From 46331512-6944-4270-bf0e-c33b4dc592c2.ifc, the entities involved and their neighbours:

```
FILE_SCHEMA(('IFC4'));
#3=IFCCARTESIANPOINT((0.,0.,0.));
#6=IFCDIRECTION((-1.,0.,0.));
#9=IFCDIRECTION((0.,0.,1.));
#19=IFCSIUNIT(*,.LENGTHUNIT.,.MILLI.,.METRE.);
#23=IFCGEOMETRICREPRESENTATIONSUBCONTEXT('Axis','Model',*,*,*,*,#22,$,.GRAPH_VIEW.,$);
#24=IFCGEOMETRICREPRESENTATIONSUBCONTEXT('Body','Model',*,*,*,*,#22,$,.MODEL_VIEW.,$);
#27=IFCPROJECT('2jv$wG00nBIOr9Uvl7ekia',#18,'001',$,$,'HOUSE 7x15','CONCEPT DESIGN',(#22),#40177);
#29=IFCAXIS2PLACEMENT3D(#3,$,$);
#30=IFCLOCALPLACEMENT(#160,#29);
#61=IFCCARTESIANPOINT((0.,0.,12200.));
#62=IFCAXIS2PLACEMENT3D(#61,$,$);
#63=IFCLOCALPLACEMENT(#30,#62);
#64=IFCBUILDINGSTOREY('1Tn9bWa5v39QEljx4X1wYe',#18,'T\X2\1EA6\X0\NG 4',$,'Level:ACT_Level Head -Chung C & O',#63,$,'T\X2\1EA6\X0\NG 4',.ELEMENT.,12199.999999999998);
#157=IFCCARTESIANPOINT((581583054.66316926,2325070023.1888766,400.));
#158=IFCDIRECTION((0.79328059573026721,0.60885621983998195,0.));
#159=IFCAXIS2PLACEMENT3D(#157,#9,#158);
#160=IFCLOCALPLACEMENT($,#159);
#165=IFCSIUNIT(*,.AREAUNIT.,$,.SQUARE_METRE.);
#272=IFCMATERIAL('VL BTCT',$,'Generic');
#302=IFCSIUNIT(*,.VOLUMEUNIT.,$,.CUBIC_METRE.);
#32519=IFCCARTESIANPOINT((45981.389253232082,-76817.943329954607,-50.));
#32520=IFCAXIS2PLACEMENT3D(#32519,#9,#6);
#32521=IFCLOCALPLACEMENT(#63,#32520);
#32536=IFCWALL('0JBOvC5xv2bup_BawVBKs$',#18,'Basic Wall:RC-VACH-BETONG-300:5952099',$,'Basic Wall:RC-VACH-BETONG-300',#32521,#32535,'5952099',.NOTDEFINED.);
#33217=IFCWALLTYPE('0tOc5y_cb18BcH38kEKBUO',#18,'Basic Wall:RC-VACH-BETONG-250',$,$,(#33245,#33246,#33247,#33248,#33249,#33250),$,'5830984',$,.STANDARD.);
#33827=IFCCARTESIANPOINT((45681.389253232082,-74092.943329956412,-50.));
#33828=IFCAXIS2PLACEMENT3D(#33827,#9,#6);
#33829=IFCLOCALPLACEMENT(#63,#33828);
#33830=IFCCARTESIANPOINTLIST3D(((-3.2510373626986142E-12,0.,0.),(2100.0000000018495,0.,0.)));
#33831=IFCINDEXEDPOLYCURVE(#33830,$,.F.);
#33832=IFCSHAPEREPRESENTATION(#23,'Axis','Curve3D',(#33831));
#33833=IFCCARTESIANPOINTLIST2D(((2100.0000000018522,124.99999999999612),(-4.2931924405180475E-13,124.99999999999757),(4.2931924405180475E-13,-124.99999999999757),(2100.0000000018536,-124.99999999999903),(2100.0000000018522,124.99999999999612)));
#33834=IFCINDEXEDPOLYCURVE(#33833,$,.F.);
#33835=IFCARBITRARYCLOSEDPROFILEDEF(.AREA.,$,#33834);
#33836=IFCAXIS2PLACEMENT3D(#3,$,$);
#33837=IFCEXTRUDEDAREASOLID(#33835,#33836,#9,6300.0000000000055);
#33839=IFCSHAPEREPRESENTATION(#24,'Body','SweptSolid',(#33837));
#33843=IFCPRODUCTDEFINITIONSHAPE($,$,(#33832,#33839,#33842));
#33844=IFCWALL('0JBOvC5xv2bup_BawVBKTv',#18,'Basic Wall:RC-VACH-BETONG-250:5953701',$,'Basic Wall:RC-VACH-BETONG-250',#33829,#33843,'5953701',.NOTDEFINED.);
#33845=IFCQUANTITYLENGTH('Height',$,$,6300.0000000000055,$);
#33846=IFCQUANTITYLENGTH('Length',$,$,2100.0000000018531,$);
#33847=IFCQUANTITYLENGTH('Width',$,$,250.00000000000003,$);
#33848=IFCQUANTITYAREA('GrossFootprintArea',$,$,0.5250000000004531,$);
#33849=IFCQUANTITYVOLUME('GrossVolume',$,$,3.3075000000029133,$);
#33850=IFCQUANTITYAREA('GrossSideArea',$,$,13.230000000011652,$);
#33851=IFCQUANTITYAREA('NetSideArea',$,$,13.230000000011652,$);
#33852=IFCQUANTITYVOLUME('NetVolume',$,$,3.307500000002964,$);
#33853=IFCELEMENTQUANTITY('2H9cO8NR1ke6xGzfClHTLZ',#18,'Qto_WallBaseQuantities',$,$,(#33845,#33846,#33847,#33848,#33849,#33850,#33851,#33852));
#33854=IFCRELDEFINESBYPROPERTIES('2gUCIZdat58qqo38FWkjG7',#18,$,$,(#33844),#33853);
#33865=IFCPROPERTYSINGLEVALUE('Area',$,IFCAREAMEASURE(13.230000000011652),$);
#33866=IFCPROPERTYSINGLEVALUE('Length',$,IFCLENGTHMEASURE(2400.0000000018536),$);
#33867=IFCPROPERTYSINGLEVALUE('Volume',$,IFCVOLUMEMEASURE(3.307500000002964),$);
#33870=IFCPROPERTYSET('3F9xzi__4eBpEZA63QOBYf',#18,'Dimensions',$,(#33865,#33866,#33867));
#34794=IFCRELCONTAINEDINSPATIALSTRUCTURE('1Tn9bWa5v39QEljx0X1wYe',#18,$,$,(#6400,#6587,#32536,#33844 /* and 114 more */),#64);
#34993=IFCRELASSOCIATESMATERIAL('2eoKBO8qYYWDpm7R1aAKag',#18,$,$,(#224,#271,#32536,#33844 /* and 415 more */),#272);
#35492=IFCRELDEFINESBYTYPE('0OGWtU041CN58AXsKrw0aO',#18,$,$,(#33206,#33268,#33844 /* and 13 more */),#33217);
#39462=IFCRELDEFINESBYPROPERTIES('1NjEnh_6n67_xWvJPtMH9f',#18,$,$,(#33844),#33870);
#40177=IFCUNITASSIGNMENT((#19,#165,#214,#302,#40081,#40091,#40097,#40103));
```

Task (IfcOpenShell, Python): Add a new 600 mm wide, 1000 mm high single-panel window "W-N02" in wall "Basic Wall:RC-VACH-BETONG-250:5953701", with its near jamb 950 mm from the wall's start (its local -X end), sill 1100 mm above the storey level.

```python
import numpy as np
import ifcopenshell
import ifcopenshell.api.feature
import ifcopenshell.api.geometry
import ifcopenshell.api.pset
import ifcopenshell.api.root
import ifcopenshell.api.spatial
import ifcopenshell.geom
import ifcopenshell.util.element
import ifcopenshell.util.placement
import ifcopenshell.util.representation
import ifcopenshell.util.shape
import ifcopenshell.util.unit

model = ifcopenshell.open("46331512-6944-4270-bf0e-c33b4dc592c2.ifc")
unit_scale = ifcopenshell.util.unit.calculate_unit_scale(model)
area_scale = ifcopenshell.util.unit.calculate_unit_scale(model, "AREAUNIT")
volume_scale = ifcopenshell.util.unit.calculate_unit_scale(model, "VOLUMEUNIT")
settings = ifcopenshell.geom.settings()


def volume(element):
    """Net volume in cubic metres, openings subtracted."""
    shape = ifcopenshell.geom.create_shape(settings, element)
    return ifcopenshell.util.shape.get_volume(shape.geometry)


wall = model.by_id(33844)
storey = ifcopenshell.util.element.get_container(wall, ifc_class="IfcBuildingStorey")
context = ifcopenshell.util.representation.get_context(model, "Model", "Body", "MODEL_VIEW")
before = volume(wall)

width, height, from_end, sill = 0.6, 1, 0.95, 1.1  # metres

# The wall runs along its own X axis, and the end named is its -X end.
wall_shape = ifcopenshell.geom.create_shape(settings, wall)
x, y, z = ifcopenshell.util.shape.get_vertices(wall_shape.geometry).T
start = x.min() + from_end
face, thickness = float(y.min()), float(y.max() - y.min())
wall_matrix = ifcopenshell.util.placement.get_local_placement(wall.ObjectPlacement)
level = ifcopenshell.util.placement.get_local_placement(storey.ObjectPlacement)[2, 3]


def in_wall(x, y):
    """Placement at x, y metres in the wall's axes, at sill height."""
    matrix = wall_matrix.copy()
    matrix[:, 3] = wall_matrix @ np.array([x / unit_scale, y / unit_scale, 0.0, 1.0])
    matrix[2, 3] = level + sill / unit_scale
    return matrix


# Opening: a box that overshoots both wall faces by 50 mm.
opening = ifcopenshell.api.root.create_entity(model, ifc_class="IfcOpeningElement", predefined_type="OPENING")
box = ifcopenshell.api.geometry.add_wall_representation(
    model, context=context, length=width, height=height, thickness=thickness + 0.1
)
ifcopenshell.api.geometry.assign_representation(model, product=opening, representation=box)
ifcopenshell.api.geometry.edit_object_placement(model, product=opening, matrix=in_wall(start, face - 0.05), is_si=False)
ifcopenshell.api.feature.add_feature(model, feature=opening, element=wall)

window = ifcopenshell.api.root.create_entity(model, ifc_class="IfcWindow", name="W-N02", predefined_type="WINDOW")
window.OverallWidth, window.OverallHeight = width / unit_scale, height / unit_scale
window.PartitioningType = "SINGLE_PANEL"
body = ifcopenshell.api.geometry.add_window_representation(
    model,
    context=context,
    overall_width=window.OverallWidth,
    overall_height=window.OverallHeight,
    partition_type="SINGLE_PANEL",
)
ifcopenshell.api.geometry.assign_representation(model, product=window, representation=body)
ifcopenshell.api.spatial.assign_container(model, products=[window], relating_structure=storey)
ifcopenshell.api.feature.add_filling(model, opening=opening, element=window)

# Centre the window in the wall's thickness.
ifcopenshell.api.geometry.edit_object_placement(model, product=window, matrix=in_wall(start, face), is_si=False)
window_shape = ifcopenshell.geom.create_shape(settings, window)
depth = ifcopenshell.util.shape.get_vertices(window_shape.geometry)[:, 1]
offset = face + thickness / 2 - (depth.min() + depth.max()) / 2
ifcopenshell.api.geometry.edit_object_placement(model, product=window, matrix=in_wall(start, offset), is_si=False)

after = volume(wall)

# Update the wall's stored quantities.
qto = model.by_id(ifcopenshell.util.element.get_pset(wall, "Qto_WallBaseQuantities", should_inherit=False)["id"])
ifcopenshell.api.pset.edit_qto(model, qto=qto, properties={
    "NetSideArea": after / thickness / area_scale,
    "NetVolume": after / volume_scale,
})
pset = model.by_id(ifcopenshell.util.element.get_pset(wall, "Dimensions", should_inherit=False)["id"])
ifcopenshell.api.pset.edit_pset(model, pset=pset, properties={
    "Area": model.create_entity("IfcAreaMeasure", after / thickness / area_scale),
    "Volume": model.create_entity("IfcVolumeMeasure", after / volume_scale),
})

print(f"wall volume {before:.3f} -> {after:.3f} m3")

model.write("46331512-6944-4270-bf0e-c33b4dc592c2_edited.ifc")
```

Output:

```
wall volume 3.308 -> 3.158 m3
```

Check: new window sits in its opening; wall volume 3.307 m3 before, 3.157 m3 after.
